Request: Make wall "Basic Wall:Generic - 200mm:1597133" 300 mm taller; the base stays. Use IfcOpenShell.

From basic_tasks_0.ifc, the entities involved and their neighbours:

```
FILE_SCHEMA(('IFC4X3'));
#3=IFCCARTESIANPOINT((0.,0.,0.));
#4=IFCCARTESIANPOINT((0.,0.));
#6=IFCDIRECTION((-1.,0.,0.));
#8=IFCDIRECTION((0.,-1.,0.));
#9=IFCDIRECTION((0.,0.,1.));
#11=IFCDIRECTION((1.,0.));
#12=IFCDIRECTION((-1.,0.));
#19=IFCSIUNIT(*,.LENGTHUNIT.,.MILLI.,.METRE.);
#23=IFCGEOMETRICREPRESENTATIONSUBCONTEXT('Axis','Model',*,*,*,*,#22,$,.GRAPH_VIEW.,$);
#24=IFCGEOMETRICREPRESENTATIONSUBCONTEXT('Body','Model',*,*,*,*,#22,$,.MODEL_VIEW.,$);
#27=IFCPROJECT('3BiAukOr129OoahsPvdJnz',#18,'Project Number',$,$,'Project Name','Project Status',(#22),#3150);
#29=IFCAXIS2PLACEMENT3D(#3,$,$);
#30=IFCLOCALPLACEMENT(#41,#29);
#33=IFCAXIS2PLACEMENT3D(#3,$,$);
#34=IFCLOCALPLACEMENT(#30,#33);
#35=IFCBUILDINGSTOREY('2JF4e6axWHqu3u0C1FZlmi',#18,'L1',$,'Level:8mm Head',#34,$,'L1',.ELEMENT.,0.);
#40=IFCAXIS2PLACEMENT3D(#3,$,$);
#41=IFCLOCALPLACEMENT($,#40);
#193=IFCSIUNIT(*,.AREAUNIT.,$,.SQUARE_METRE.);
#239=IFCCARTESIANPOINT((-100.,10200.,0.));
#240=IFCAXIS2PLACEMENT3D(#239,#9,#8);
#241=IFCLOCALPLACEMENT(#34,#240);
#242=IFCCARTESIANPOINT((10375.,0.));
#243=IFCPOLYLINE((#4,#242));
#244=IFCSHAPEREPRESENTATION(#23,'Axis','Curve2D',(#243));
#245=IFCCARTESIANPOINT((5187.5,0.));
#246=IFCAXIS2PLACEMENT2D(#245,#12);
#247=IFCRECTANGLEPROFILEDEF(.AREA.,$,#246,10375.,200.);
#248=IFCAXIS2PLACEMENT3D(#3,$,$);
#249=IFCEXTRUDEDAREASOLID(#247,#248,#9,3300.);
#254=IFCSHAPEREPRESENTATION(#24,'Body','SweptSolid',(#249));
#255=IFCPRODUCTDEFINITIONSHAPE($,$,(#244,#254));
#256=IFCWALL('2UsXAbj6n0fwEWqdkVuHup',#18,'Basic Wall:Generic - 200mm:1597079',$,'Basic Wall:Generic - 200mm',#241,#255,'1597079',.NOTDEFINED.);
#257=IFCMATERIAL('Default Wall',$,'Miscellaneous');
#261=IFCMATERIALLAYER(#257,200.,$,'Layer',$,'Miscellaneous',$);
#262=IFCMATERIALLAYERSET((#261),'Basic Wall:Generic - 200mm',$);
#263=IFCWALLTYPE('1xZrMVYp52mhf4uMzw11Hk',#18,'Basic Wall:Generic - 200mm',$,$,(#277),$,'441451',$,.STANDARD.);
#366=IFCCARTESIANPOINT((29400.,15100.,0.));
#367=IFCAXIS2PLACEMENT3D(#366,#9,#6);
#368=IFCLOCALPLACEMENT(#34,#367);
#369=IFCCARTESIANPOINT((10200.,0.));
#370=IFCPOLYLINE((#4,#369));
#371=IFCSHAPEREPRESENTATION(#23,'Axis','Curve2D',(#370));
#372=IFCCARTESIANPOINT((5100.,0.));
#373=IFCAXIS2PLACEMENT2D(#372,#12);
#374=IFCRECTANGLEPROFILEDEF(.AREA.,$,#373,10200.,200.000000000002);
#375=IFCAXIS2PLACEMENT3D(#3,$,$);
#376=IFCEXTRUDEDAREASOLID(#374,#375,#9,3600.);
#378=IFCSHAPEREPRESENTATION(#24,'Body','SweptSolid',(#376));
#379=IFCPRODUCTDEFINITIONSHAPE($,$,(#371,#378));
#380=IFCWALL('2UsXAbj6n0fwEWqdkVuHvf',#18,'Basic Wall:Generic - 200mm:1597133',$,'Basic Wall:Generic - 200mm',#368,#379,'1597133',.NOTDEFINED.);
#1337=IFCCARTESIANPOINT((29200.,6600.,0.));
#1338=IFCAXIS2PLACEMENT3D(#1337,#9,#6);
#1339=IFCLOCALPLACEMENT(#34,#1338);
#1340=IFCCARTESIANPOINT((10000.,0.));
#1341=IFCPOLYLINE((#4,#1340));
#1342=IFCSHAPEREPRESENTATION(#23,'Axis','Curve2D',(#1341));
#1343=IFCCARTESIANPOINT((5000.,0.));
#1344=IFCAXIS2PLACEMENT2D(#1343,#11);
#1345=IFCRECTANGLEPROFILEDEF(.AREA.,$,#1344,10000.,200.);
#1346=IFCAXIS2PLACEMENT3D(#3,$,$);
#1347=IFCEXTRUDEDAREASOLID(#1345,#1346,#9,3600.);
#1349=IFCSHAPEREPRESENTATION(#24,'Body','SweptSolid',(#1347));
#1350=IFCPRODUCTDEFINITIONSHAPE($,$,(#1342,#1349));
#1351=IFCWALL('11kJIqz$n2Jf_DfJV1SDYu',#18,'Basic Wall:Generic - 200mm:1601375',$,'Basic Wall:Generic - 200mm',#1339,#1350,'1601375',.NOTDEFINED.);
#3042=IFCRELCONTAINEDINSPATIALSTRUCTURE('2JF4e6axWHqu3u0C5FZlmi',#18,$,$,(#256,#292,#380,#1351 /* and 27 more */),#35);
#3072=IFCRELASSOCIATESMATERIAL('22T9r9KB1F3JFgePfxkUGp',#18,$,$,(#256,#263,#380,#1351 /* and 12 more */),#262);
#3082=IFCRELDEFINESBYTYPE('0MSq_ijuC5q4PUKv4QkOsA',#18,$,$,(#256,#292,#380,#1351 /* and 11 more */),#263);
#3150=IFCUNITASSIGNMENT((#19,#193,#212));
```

```python
import ifcopenshell
import ifcopenshell.geom
import ifcopenshell.util.representation
import ifcopenshell.util.shape
import ifcopenshell.util.unit

model = ifcopenshell.open("basic_tasks_0.ifc")
unit_scale = ifcopenshell.util.unit.calculate_unit_scale(model)
settings = ifcopenshell.geom.settings()


def volume(element):
    """Net volume in cubic metres, openings subtracted."""
    shape = ifcopenshell.geom.create_shape(settings, element)
    return ifcopenshell.util.shape.get_volume(shape.geometry)


wall = model.by_guid("2UsXAbj6n0fwEWqdkVuHvf")
before = volume(wall)

body = ifcopenshell.util.representation.get_representation(wall, "Model", "Body")
solid = body.Items[0]
old_height = solid.Depth
solid.Depth += 0.3 / unit_scale
after = volume(wall)

print(f"height {old_height:g} -> {solid.Depth:g}, volume {before:.3f} -> {after:.3f} m3")

model.write("basic_tasks_0_edited.ifc")
```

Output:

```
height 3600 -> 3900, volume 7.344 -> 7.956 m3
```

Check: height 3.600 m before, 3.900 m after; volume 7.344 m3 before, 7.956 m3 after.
